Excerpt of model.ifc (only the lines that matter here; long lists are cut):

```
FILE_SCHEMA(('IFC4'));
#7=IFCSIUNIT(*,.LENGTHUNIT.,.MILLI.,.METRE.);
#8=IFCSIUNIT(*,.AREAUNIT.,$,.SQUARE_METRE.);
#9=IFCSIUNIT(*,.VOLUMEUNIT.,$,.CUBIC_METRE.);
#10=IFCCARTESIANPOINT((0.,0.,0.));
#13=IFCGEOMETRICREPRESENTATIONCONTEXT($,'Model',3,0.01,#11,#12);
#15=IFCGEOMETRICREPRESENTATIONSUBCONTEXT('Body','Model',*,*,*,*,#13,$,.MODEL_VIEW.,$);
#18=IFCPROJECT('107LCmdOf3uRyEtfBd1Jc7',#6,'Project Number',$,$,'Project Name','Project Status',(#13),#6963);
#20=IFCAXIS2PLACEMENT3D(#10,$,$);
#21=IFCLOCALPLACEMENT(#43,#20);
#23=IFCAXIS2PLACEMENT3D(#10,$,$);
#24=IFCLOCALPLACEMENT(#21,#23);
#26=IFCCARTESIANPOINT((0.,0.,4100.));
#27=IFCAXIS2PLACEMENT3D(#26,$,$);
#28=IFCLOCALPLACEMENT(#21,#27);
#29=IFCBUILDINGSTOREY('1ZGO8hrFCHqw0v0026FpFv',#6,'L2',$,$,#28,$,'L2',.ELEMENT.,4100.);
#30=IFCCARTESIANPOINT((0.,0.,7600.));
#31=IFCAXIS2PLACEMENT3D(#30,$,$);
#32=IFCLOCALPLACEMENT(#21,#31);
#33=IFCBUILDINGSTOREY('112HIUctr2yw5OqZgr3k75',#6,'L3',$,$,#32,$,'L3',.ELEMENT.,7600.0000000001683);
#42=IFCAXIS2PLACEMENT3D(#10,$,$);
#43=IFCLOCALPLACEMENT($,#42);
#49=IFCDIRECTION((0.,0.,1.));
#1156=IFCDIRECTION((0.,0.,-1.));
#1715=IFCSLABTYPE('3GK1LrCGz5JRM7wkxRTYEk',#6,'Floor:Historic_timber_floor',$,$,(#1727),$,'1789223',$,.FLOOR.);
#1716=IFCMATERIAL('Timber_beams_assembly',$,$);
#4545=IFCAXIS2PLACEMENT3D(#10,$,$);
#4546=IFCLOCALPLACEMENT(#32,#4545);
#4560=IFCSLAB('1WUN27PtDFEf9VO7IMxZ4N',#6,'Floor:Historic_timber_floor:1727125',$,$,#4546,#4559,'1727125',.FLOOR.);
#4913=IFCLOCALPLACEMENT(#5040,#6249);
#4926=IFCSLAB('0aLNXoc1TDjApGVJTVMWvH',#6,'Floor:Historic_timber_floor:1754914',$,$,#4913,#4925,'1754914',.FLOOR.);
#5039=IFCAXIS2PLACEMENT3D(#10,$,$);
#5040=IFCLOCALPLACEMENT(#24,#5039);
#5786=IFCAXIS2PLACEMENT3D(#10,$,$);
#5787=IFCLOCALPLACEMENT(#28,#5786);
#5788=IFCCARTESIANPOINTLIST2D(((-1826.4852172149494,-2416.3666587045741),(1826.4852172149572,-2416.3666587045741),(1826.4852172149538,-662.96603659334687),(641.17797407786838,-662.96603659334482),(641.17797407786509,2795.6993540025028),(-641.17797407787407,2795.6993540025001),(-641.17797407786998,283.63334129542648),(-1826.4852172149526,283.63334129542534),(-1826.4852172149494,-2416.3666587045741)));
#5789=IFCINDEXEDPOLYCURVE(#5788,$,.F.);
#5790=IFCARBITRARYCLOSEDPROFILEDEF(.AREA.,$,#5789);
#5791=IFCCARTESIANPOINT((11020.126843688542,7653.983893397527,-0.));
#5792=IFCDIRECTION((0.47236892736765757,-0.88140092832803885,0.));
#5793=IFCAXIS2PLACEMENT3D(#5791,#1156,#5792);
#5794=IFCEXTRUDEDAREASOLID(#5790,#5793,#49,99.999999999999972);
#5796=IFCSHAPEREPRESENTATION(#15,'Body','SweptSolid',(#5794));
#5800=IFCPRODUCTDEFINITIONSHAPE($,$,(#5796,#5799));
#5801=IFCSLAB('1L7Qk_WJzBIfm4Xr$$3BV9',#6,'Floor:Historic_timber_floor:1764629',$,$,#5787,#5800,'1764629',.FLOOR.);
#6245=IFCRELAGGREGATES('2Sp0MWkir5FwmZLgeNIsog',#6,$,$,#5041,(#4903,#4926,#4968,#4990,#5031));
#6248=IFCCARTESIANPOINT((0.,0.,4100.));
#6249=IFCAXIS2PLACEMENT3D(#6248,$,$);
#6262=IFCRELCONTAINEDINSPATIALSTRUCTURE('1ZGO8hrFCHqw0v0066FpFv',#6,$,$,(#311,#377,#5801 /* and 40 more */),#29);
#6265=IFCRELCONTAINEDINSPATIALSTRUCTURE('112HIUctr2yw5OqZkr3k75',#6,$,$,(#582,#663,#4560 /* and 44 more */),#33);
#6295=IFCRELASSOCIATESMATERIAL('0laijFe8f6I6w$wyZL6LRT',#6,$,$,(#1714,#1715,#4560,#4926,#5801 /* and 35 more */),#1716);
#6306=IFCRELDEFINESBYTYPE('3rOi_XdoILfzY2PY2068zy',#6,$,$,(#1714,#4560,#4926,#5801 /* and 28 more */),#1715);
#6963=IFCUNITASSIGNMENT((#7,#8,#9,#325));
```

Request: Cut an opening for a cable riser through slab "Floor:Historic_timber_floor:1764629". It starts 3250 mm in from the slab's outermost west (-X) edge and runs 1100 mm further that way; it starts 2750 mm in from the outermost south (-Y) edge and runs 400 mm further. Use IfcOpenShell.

```python
import numpy as np
import ifcopenshell
import ifcopenshell.api.feature
import ifcopenshell.api.geometry
import ifcopenshell.api.root
import ifcopenshell.geom
import ifcopenshell.util.placement
import ifcopenshell.util.representation
import ifcopenshell.util.shape
import ifcopenshell.util.unit

model = ifcopenshell.open("model.ifc")
unit_scale = ifcopenshell.util.unit.calculate_unit_scale(model)
settings = ifcopenshell.geom.settings()


def volume(element):
    """Net volume in cubic metres, openings subtracted."""
    shape = ifcopenshell.geom.create_shape(settings, element)
    return ifcopenshell.util.shape.get_volume(shape.geometry)


slab = model.by_guid("1L7Qk_WJzBIfm4Xr$$3BV9")
before = volume(slab)

# Extent in the slab's own axes, in metres. The edges named are its -X and -Y sides.
slab_shape = ifcopenshell.geom.create_shape(settings, slab)
vertices = ifcopenshell.util.shape.get_vertices(slab_shape.geometry)
x_min, y_min, bottom = vertices.min(axis=0)
top = vertices[:, 2].max()

opening = ifcopenshell.api.root.create_entity(model, ifc_class="IfcOpeningElement", name="Cable riser opening", predefined_type="OPENING")
context = ifcopenshell.util.representation.get_context(model, "Model", "Body", "MODEL_VIEW")
width, depth = 1.1, 0.4
outline = [(0.0, 0.0), (width, 0.0), (width, depth), (0.0, depth), (0.0, 0.0)]
# Overshoot both faces by 50 mm so the cut is clean.
shape = ifcopenshell.api.geometry.add_slab_representation(
    model, context=context, depth=top - bottom + 0.1, polyline=outline
)
ifcopenshell.api.geometry.assign_representation(model, product=opening, representation=shape)

matrix = ifcopenshell.util.placement.get_local_placement(slab.ObjectPlacement)
matrix[:, 3] = matrix @ np.append(np.array([x_min + 3.25, y_min + 2.75, bottom - 0.05]) / unit_scale, 1.0)
ifcopenshell.api.geometry.edit_object_placement(model, product=opening, matrix=matrix, is_si=False)
ifcopenshell.api.feature.add_feature(model, feature=opening, element=slab)

after = volume(slab)

print(f"slab volume {before:.3f} -> {after:.3f} m3")

model.write("model-out.ifc")
```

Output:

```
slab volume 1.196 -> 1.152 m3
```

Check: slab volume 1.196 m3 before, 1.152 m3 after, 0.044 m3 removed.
